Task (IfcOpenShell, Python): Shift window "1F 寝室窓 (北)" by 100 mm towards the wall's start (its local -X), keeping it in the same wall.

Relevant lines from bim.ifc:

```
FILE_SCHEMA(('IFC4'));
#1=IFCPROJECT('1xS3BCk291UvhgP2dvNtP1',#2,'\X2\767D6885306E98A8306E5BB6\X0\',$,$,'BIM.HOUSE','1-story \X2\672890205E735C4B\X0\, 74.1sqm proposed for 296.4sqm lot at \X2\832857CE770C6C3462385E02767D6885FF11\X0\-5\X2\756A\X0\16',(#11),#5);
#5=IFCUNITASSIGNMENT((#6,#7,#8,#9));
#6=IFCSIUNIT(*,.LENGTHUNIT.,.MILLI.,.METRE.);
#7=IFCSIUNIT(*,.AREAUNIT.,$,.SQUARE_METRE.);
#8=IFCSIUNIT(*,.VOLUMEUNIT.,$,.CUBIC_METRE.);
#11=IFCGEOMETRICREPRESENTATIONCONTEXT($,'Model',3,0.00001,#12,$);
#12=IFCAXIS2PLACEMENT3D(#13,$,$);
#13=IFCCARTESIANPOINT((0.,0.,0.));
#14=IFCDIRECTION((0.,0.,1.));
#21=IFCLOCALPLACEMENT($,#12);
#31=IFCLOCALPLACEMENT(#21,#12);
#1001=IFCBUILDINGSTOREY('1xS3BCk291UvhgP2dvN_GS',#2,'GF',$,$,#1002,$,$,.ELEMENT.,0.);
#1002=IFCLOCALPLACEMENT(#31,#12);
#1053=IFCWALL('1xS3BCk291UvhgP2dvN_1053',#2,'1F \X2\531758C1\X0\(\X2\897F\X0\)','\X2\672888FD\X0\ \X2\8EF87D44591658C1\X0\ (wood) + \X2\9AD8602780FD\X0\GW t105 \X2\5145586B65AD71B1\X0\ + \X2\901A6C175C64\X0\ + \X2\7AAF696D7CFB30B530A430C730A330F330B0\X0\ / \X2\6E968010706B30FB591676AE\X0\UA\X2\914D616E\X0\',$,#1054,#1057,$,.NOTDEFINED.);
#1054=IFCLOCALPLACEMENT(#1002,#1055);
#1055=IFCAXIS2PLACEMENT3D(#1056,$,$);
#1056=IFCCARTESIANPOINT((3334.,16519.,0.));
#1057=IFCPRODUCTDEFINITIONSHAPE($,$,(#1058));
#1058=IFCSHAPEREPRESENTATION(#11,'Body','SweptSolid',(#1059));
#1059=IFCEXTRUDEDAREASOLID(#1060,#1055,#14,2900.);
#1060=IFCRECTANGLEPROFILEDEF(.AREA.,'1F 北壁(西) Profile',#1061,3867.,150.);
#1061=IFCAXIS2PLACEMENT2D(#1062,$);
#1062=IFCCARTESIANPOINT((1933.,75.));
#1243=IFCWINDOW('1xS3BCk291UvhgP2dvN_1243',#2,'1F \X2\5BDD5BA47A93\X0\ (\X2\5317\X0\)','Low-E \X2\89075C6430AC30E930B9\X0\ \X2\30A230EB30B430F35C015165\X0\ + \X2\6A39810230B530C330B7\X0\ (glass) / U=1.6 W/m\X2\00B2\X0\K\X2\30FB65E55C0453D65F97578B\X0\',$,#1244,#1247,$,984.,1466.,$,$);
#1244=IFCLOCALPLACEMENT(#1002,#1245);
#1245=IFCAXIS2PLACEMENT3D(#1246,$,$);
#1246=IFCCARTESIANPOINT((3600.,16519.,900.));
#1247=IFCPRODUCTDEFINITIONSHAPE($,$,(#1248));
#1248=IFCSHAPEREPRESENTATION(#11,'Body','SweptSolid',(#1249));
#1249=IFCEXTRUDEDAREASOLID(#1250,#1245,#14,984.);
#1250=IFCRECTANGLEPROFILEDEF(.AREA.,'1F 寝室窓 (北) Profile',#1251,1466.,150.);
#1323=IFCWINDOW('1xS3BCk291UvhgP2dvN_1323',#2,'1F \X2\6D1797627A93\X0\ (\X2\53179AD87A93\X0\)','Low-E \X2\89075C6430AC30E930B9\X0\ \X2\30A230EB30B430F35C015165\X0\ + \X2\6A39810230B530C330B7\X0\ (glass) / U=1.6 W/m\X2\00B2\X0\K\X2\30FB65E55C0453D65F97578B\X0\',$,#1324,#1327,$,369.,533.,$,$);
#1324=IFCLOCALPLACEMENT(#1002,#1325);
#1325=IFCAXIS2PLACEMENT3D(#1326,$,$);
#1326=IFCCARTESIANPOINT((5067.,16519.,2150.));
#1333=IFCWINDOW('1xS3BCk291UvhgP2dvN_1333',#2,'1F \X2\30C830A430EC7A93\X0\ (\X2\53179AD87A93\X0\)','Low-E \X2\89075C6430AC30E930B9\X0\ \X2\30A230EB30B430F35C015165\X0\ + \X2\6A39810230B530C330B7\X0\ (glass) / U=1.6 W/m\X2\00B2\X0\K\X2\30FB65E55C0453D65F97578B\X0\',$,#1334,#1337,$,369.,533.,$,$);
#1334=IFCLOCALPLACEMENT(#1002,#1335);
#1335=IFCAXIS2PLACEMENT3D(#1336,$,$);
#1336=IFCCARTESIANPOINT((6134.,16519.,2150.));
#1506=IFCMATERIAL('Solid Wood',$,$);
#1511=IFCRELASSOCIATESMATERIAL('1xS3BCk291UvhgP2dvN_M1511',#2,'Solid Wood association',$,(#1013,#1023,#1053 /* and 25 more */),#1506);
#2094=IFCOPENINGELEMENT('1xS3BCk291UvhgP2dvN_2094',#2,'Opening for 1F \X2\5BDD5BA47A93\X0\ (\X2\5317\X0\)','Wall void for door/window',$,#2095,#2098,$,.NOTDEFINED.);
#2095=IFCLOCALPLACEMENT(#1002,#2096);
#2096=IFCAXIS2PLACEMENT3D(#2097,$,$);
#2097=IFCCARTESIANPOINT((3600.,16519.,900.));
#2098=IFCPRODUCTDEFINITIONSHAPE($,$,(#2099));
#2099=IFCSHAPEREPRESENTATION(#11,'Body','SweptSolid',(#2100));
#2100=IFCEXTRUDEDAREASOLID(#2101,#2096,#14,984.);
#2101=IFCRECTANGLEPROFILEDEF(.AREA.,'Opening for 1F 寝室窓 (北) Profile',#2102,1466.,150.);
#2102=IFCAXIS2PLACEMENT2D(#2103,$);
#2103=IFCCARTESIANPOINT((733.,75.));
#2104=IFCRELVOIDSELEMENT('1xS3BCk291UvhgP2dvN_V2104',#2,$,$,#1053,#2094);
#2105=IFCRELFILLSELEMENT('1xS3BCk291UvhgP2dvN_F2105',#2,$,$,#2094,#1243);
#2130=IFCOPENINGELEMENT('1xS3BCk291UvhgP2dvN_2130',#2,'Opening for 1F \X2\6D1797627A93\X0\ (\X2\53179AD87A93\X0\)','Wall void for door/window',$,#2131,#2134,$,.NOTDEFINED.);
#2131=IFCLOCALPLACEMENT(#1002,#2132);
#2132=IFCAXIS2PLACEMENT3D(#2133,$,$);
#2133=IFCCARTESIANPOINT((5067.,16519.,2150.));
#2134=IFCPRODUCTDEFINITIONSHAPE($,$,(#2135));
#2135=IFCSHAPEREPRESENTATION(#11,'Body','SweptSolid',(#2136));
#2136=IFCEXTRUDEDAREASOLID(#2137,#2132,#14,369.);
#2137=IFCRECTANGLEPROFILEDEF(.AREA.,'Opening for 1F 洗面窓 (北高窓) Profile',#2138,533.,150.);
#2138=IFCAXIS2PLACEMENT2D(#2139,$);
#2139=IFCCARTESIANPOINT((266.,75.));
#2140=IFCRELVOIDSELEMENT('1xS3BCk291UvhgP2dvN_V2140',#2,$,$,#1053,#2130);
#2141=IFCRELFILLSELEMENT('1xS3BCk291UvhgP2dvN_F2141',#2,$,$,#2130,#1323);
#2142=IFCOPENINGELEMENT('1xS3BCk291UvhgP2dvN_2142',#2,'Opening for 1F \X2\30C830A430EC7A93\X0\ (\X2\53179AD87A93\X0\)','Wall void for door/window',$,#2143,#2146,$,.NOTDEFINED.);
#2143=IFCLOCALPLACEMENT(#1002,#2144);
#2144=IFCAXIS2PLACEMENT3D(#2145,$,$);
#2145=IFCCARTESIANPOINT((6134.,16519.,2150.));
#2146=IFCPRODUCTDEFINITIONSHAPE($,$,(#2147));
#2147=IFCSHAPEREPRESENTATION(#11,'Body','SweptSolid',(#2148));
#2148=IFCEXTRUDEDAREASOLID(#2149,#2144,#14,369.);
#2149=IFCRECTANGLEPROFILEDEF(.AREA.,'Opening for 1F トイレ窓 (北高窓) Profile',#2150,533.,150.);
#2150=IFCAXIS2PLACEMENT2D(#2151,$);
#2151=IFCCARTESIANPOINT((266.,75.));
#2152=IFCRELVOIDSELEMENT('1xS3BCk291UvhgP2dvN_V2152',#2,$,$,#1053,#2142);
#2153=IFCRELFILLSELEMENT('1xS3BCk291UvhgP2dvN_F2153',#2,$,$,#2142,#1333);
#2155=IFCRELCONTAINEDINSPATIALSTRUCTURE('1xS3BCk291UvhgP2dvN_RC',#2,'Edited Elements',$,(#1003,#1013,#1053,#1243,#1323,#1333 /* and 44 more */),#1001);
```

```python
import ifcopenshell
import ifcopenshell.api.geometry
import ifcopenshell.util.placement
import ifcopenshell.util.unit

model = ifcopenshell.open("bim.ifc")
unit_scale = ifcopenshell.util.unit.calculate_unit_scale(model)

window = model.by_id(1243)
opening = window.FillsVoids[0].RelatingOpeningElement
wall = opening.VoidsElements[0].RelatingBuildingElement

wall_matrix = ifcopenshell.util.placement.get_local_placement(wall.ObjectPlacement)
shift = wall_matrix[:3, 0] * -0.1 / unit_scale
before = ifcopenshell.util.placement.get_local_placement(window.ObjectPlacement)[:3, 3].copy()

# The window is not placed relative to its opening, so move both.
for product in (opening, window):
    matrix = ifcopenshell.util.placement.get_local_placement(product.ObjectPlacement)
    matrix[:3, 3] += shift
    ifcopenshell.api.geometry.edit_object_placement(model, product=product, matrix=matrix, is_si=False)

after = ifcopenshell.util.placement.get_local_placement(window.ObjectPlacement)[:3, 3]
print("window moved by", (after - before).round(3) + 0.0)

model.write("bim_rev.ifc")
```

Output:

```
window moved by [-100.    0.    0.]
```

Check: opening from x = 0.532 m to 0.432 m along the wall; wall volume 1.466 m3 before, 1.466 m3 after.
